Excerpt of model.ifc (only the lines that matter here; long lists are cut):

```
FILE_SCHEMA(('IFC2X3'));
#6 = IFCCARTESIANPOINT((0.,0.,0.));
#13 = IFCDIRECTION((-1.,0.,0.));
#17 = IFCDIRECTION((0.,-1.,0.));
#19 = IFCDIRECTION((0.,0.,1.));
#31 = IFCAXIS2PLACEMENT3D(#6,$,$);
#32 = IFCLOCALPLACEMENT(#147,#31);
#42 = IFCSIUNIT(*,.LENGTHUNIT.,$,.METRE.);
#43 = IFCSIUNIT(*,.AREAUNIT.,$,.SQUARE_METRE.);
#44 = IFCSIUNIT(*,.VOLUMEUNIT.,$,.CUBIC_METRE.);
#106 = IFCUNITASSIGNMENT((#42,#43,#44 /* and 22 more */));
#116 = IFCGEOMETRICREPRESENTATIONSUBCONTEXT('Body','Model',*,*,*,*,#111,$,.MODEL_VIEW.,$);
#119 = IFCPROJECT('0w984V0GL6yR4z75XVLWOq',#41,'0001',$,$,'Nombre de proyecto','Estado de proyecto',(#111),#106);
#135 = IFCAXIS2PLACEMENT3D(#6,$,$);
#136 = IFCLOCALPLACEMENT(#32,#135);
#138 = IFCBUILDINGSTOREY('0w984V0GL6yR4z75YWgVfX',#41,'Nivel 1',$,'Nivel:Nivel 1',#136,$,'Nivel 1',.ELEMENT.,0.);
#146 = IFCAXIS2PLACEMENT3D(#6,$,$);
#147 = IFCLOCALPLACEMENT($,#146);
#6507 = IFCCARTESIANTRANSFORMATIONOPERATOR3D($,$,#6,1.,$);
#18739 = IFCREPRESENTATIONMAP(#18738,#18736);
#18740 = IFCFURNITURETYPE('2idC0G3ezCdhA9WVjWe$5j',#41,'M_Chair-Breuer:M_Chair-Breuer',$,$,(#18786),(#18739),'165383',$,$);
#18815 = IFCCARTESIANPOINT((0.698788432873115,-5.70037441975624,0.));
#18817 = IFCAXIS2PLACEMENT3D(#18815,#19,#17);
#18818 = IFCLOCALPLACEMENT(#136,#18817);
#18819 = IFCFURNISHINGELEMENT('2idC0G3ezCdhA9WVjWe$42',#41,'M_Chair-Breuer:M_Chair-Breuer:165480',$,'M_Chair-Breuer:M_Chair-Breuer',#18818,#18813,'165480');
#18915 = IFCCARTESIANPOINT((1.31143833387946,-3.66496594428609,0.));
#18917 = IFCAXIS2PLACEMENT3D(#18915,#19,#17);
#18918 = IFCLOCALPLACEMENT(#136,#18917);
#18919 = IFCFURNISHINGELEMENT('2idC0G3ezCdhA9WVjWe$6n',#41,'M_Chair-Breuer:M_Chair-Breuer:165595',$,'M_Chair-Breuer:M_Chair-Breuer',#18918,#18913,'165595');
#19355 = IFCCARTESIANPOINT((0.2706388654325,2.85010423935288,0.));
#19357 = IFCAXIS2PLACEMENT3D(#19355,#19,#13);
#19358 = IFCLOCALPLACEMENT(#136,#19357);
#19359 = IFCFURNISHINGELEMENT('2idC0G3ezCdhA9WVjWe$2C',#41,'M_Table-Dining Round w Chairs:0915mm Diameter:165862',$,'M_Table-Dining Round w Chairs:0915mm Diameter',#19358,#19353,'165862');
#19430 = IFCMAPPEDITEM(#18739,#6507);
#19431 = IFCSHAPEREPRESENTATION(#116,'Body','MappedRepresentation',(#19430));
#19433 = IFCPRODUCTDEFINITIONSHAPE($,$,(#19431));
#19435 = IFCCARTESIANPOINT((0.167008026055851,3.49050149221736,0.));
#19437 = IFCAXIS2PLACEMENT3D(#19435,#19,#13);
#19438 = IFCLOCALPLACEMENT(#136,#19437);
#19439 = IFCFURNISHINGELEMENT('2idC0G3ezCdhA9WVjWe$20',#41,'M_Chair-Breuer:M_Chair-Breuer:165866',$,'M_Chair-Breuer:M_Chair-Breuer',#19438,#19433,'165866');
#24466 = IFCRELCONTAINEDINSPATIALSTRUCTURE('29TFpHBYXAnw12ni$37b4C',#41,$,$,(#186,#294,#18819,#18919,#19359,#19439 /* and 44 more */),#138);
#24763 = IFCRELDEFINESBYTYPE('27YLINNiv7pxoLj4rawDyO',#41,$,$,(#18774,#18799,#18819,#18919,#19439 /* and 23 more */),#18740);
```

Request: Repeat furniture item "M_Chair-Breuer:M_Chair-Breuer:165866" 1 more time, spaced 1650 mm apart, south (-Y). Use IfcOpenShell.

```python
import numpy as np
import ifcopenshell
import ifcopenshell.api.geometry
import ifcopenshell.api.root
import ifcopenshell.util.element
import ifcopenshell.util.placement

model = ifcopenshell.open("model.ifc")


def reuse_history(source, copy):
    """copy_class also copies each property set's owner history, people and application; keep the originals."""
    for rel in copy.IsDefinedBy:
        if rel.is_a("IfcRelDefinesByProperties") and (history := rel.RelatingPropertyDefinition.OwnerHistory):
            rel.RelatingPropertyDefinition.OwnerHistory = source.OwnerHistory
            ifcopenshell.util.element.remove_deep2(model, history)


source = model.by_id(19439)
base = ifcopenshell.util.placement.get_local_placement(source.ObjectPlacement)
step = np.array([0.0, -1.0, 0.0]) * 1.65

for i in range(1, 2):
    copy = ifcopenshell.api.root.copy_class(model, product=source)
    copy.Representation = ifcopenshell.util.element.copy_deep(
        model, source.Representation, exclude=["IfcGeometricRepresentationContext", "IfcRepresentationMap"]
    )
    copy.Name = "M_Chair-Breuer:M_Chair-Breuer"
    copy.Tag = None
    reuse_history(source, copy)
    matrix = base.copy()
    matrix[:3, 3] += i * step
    print("added at", matrix[:3, 3].round(3) + 0.0)
    ifcopenshell.api.geometry.edit_object_placement(model, product=copy, matrix=matrix, is_si=False)

model.write("model_updated.ifc")
```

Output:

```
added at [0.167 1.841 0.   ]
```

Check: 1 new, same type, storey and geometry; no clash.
